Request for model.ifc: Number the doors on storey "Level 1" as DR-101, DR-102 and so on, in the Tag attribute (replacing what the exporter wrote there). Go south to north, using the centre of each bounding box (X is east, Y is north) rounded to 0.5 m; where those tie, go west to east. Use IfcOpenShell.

First a look at what the model holds.

```python
import ifcopenshell
import ifcopenshell.util.element
import ifcopenshell.util.placement

model = ifcopenshell.open("model.ifc")
print(model.schema)
storey = next(s for s in model.by_type("IfcBuildingStorey") if s.Name == "Level 1")
doors = [e for e in ifcopenshell.util.element.get_decomposition(storey) if e.is_a("IfcDoor")]
for e in sorted(doors, key=lambda e: e.id()):
    origin = ifcopenshell.util.placement.get_local_placement(e.ObjectPlacement)[:3, 3]
    print(e.id(), e.Tag, e.Name, origin.round(2) + 0.0, sep=" | ")
```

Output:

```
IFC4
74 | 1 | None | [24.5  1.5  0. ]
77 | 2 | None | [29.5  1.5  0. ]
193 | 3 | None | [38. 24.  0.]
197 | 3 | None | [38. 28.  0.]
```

```python
import ifcopenshell
import ifcopenshell.geom
import ifcopenshell.util.element
import ifcopenshell.util.shape

model = ifcopenshell.open("model.ifc")
settings = ifcopenshell.geom.settings()
settings.set("use-world-coords", True)


def centre(element):
    shape = ifcopenshell.geom.create_shape(settings, element)
    return ifcopenshell.util.shape.get_bbox_centroid(shape.geometry)


storey = next(s for s in model.by_type("IfcBuildingStorey") if s.Name == "Level 1")
doors = [e for e in ifcopenshell.util.element.get_decomposition(storey) if e.is_a("IfcDoor")]

# Insertion points can sit at a corner or the storey origin, so sort by the geometry (in metres).
centres = {e: centre(e) for e in doors}
doors.sort(key=lambda e: (round(centres[e][1] / 0.5), centres[e][0]))

for i, e in enumerate(doors, start=1):
    number = f"DR-1{i:02d}"
    e.Tag = number
    print(e.id(), number)

model.write("model_rev.ifc")
```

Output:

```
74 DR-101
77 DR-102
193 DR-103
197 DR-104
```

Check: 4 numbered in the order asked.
